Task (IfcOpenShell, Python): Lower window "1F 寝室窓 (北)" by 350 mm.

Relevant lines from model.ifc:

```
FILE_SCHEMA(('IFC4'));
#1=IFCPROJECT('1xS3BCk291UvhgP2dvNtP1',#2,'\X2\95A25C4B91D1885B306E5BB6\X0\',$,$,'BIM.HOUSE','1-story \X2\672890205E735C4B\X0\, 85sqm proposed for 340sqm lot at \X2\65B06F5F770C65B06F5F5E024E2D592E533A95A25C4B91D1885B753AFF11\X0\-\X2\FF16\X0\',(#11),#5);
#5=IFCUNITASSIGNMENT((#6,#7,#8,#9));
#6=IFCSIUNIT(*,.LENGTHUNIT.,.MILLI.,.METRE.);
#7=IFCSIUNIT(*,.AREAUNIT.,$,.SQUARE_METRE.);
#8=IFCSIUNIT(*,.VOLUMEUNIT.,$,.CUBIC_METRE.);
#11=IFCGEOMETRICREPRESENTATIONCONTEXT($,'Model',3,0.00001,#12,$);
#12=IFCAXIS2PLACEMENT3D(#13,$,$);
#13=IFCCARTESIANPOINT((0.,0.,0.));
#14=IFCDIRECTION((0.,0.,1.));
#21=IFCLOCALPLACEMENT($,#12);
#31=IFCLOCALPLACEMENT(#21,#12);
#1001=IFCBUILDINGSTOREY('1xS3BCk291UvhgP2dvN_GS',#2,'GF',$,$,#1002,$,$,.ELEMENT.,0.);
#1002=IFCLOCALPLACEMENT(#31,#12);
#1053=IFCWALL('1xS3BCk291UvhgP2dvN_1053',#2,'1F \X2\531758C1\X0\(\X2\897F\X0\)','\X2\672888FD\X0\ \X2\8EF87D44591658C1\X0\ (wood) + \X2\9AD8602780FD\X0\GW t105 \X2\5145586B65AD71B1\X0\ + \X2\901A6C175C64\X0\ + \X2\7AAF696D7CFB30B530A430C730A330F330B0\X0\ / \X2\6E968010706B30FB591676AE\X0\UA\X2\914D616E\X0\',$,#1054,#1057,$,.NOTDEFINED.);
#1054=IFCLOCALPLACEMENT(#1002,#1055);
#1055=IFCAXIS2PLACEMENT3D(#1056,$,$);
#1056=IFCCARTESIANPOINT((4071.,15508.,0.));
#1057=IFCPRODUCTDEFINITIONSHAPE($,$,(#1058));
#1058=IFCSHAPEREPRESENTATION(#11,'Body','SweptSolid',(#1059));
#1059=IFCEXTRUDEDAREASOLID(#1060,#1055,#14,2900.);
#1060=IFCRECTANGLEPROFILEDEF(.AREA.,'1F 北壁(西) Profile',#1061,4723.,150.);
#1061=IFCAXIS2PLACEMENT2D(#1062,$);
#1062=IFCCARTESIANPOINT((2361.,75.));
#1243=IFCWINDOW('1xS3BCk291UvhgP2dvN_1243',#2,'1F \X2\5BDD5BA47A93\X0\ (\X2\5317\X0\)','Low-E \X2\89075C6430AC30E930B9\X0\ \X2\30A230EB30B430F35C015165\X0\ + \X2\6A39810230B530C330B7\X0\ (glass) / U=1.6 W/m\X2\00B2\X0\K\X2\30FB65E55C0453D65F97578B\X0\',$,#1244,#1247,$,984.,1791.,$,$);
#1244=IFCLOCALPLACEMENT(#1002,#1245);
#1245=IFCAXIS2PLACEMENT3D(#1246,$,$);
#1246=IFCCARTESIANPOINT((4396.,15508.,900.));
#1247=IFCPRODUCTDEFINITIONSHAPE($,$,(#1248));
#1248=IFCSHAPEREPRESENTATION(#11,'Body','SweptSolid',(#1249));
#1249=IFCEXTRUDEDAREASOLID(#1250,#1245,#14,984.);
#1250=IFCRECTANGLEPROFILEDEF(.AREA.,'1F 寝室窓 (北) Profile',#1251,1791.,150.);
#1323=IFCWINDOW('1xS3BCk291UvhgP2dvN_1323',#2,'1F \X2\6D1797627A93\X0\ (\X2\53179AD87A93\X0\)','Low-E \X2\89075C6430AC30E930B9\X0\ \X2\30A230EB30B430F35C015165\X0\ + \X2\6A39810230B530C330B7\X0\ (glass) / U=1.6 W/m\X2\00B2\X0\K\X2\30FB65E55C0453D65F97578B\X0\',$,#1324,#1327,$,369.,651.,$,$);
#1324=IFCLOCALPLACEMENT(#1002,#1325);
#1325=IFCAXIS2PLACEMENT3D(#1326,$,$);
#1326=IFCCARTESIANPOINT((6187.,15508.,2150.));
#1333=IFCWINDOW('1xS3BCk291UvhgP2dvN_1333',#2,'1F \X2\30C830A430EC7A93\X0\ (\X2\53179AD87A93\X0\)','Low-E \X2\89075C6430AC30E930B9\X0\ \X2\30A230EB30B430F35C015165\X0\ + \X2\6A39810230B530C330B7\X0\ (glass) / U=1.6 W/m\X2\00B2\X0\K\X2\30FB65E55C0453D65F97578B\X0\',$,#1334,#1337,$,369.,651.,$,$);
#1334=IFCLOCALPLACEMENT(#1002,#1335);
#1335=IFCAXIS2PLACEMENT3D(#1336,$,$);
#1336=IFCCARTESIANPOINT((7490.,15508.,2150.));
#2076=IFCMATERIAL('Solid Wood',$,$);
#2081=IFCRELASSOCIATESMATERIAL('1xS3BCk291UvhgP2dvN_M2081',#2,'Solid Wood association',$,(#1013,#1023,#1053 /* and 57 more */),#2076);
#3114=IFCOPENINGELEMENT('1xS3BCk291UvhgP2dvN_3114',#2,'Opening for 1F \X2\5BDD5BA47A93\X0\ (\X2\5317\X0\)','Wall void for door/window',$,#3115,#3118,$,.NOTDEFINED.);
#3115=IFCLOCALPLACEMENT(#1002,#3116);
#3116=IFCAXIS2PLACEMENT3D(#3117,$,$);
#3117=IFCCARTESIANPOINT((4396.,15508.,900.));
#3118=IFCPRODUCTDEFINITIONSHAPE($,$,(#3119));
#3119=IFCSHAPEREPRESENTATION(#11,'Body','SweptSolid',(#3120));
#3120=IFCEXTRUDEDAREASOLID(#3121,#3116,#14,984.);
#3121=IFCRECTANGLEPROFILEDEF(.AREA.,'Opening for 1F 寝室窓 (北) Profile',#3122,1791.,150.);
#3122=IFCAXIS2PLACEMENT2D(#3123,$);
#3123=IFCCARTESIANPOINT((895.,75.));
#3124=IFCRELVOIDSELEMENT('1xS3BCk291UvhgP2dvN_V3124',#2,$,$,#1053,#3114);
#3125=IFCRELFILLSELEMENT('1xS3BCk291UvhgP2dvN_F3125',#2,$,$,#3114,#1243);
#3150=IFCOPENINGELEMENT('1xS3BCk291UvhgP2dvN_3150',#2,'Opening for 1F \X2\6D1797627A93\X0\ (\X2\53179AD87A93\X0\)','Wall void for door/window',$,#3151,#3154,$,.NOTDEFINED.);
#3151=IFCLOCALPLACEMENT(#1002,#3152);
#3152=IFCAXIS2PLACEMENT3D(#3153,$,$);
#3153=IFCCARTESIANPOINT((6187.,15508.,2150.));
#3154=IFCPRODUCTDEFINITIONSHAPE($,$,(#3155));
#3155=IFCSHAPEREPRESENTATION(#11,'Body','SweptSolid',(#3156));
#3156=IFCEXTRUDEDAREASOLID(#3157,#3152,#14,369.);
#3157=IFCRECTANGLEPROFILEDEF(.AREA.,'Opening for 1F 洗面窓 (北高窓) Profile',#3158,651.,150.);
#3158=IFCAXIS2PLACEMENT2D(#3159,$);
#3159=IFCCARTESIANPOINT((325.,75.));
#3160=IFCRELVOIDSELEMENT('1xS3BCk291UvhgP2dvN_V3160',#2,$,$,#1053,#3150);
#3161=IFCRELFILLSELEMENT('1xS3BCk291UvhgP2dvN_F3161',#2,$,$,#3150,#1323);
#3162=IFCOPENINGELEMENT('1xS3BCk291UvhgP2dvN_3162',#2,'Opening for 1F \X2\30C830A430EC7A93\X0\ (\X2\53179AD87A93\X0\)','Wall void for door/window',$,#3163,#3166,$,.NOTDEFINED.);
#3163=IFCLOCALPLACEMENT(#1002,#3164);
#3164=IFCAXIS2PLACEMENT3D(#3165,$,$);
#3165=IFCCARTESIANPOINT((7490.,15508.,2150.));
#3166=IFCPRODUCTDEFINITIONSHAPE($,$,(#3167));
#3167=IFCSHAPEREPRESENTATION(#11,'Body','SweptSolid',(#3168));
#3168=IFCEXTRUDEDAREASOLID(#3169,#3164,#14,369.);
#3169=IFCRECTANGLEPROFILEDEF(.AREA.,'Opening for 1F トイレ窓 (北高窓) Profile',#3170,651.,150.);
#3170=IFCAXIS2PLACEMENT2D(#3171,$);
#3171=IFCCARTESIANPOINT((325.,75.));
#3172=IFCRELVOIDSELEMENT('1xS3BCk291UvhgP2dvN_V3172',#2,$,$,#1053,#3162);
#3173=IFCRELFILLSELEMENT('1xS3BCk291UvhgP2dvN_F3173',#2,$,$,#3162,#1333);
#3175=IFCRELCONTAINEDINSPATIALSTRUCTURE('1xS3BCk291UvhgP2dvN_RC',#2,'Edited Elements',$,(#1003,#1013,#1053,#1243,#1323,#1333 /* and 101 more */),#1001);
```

```python
import numpy as np
import ifcopenshell
import ifcopenshell.api.geometry
import ifcopenshell.util.placement
import ifcopenshell.util.unit

model = ifcopenshell.open("model.ifc")
unit_scale = ifcopenshell.util.unit.calculate_unit_scale(model)

window = model.by_id(1243)
opening = window.FillsVoids[0].RelatingOpeningElement
dz = -350.0

shift = np.array([0.0, 0.0, dz])
# The window is not placed relative to its opening, so move both.
for product in (opening, window):
    matrix = ifcopenshell.util.placement.get_local_placement(product.ObjectPlacement)
    matrix[:3, 3] += shift
    ifcopenshell.api.geometry.edit_object_placement(model, product=product, matrix=matrix, is_si=False)

print(f"moved by {dz * unit_scale:+.3f} m")

model.write("model_edited.ifc")
```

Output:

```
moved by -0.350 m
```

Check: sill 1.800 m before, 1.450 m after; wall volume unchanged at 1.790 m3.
